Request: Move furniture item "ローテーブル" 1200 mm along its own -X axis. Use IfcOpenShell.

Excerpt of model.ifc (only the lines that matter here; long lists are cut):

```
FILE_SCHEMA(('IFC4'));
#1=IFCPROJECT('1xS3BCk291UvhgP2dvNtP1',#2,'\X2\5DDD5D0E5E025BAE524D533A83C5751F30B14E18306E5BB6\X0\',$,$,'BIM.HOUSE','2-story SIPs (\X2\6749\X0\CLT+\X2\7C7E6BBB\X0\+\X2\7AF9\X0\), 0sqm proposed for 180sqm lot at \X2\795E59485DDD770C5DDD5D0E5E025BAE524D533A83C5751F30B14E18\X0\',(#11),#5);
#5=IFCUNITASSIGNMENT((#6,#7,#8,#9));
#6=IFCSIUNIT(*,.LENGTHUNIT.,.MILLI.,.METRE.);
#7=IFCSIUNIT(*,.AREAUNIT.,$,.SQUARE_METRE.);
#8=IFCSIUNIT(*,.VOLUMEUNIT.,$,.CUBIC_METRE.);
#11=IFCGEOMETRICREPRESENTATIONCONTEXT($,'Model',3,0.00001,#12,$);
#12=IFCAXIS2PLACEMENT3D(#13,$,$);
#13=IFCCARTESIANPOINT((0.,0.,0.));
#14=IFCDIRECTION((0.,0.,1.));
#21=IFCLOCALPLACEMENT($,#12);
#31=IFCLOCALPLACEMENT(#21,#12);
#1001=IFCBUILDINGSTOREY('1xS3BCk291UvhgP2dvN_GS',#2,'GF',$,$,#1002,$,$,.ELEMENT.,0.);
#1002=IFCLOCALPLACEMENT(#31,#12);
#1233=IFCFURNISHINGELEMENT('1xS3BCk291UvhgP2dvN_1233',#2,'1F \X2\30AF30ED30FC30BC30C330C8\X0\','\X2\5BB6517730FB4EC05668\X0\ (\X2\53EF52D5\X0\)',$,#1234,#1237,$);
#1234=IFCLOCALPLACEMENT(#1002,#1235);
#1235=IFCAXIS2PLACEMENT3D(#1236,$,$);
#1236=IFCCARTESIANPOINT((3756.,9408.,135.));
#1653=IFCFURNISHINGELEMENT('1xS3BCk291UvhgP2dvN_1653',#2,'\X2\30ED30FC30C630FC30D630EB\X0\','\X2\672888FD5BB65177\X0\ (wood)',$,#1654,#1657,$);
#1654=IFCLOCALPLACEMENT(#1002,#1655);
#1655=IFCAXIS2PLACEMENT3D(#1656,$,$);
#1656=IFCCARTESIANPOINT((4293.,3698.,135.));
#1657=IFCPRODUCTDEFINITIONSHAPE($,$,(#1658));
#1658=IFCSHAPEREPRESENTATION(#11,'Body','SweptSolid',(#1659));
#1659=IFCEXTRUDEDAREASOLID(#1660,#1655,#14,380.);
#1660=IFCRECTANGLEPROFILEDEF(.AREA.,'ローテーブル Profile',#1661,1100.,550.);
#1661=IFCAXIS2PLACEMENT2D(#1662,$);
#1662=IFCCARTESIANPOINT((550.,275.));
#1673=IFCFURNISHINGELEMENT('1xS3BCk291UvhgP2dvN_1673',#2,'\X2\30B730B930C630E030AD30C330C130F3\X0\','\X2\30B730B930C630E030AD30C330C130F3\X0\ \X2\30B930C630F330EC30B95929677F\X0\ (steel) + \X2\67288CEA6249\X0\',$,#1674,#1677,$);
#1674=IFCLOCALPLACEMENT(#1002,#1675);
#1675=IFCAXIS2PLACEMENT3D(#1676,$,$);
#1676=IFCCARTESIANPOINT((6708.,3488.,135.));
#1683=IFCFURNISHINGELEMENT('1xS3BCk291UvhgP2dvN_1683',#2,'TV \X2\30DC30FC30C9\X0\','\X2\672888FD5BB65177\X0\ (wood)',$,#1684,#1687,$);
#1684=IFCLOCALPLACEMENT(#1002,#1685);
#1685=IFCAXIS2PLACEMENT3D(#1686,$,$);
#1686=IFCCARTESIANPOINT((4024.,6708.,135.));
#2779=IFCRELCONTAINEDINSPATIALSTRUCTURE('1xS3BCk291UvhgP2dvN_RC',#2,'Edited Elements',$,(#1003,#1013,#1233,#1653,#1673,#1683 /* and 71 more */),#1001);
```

```python
import ifcopenshell
import ifcopenshell.api.geometry
import ifcopenshell.util.placement

model = ifcopenshell.open("model.ifc")

item = model.by_id(1653)
matrix = ifcopenshell.util.placement.get_local_placement(item.ObjectPlacement)
matrix[:3, 3] -= matrix[:3, 0] * 1200.0
ifcopenshell.api.geometry.edit_object_placement(model, product=item, matrix=matrix, is_si=False)

print(ifcopenshell.util.placement.get_local_placement(item.ObjectPlacement).round(3) + 0.0)

model.write("model_edited.ifc")
```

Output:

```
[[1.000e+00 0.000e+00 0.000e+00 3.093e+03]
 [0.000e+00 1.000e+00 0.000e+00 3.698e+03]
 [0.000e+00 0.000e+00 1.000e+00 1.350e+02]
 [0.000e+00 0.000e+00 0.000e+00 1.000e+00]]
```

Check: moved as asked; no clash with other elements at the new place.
